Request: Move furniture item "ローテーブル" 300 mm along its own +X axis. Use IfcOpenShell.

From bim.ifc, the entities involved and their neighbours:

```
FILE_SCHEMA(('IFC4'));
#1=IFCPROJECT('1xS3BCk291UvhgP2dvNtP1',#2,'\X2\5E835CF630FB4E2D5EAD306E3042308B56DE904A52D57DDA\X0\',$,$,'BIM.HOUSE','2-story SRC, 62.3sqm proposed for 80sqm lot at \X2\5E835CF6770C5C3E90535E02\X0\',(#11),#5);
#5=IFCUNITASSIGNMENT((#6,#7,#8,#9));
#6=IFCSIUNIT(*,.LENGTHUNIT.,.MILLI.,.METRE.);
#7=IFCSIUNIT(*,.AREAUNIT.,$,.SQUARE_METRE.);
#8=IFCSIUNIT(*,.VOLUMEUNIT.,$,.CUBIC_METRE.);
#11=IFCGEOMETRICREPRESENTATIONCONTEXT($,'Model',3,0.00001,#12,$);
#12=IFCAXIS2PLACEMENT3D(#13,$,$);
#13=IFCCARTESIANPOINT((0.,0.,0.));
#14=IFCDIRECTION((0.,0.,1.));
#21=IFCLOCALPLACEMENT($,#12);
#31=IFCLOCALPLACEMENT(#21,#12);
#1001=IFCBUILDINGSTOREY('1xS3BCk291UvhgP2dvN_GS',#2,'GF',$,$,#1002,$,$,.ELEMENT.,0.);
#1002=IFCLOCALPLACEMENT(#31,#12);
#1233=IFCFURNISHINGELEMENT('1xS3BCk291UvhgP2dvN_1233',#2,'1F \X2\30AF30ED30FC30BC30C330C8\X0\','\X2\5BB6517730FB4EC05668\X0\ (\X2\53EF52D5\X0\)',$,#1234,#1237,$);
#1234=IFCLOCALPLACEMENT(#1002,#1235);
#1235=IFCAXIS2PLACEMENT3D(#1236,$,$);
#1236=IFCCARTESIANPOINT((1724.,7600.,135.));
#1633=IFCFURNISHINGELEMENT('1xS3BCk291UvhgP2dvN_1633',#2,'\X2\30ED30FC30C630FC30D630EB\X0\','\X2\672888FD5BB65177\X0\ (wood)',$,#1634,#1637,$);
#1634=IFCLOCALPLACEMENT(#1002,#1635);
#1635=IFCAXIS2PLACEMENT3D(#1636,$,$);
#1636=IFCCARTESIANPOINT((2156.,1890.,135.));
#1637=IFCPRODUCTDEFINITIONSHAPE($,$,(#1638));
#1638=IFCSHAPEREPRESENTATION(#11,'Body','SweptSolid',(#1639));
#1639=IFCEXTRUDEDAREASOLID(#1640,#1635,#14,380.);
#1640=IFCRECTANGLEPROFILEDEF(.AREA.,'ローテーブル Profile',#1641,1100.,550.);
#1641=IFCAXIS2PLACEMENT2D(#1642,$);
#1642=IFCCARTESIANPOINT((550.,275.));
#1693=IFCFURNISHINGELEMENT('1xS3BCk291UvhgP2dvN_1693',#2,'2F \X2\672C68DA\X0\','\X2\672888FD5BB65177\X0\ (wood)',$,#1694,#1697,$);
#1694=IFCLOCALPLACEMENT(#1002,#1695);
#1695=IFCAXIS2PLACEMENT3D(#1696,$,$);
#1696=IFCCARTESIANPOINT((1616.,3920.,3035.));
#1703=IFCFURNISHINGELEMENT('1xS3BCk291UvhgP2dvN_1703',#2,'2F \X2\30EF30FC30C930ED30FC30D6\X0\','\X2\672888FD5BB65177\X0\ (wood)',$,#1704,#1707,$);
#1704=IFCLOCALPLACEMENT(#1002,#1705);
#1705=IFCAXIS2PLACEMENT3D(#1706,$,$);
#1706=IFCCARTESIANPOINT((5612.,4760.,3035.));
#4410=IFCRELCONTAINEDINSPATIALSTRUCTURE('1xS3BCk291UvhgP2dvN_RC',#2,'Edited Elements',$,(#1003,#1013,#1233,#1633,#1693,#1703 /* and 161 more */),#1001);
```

```python
import ifcopenshell
import ifcopenshell.api.geometry
import ifcopenshell.util.placement
import ifcopenshell.util.unit

model = ifcopenshell.open("bim.ifc")
unit_scale = ifcopenshell.util.unit.calculate_unit_scale(model)

item = model.by_guid("1xS3BCk291UvhgP2dvN_1633")
matrix = ifcopenshell.util.placement.get_local_placement(item.ObjectPlacement)
matrix[:3, 3] += matrix[:3, 0] * 0.3 / unit_scale
ifcopenshell.api.geometry.edit_object_placement(model, product=item, matrix=matrix, is_si=False)

print(ifcopenshell.util.placement.get_local_placement(item.ObjectPlacement).round(3) + 0.0)

model.write("bim-out.ifc")
```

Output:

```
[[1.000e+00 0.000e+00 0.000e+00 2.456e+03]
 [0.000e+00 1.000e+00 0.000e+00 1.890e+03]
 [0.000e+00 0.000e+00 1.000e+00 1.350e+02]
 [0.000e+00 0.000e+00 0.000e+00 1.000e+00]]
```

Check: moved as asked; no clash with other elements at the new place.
